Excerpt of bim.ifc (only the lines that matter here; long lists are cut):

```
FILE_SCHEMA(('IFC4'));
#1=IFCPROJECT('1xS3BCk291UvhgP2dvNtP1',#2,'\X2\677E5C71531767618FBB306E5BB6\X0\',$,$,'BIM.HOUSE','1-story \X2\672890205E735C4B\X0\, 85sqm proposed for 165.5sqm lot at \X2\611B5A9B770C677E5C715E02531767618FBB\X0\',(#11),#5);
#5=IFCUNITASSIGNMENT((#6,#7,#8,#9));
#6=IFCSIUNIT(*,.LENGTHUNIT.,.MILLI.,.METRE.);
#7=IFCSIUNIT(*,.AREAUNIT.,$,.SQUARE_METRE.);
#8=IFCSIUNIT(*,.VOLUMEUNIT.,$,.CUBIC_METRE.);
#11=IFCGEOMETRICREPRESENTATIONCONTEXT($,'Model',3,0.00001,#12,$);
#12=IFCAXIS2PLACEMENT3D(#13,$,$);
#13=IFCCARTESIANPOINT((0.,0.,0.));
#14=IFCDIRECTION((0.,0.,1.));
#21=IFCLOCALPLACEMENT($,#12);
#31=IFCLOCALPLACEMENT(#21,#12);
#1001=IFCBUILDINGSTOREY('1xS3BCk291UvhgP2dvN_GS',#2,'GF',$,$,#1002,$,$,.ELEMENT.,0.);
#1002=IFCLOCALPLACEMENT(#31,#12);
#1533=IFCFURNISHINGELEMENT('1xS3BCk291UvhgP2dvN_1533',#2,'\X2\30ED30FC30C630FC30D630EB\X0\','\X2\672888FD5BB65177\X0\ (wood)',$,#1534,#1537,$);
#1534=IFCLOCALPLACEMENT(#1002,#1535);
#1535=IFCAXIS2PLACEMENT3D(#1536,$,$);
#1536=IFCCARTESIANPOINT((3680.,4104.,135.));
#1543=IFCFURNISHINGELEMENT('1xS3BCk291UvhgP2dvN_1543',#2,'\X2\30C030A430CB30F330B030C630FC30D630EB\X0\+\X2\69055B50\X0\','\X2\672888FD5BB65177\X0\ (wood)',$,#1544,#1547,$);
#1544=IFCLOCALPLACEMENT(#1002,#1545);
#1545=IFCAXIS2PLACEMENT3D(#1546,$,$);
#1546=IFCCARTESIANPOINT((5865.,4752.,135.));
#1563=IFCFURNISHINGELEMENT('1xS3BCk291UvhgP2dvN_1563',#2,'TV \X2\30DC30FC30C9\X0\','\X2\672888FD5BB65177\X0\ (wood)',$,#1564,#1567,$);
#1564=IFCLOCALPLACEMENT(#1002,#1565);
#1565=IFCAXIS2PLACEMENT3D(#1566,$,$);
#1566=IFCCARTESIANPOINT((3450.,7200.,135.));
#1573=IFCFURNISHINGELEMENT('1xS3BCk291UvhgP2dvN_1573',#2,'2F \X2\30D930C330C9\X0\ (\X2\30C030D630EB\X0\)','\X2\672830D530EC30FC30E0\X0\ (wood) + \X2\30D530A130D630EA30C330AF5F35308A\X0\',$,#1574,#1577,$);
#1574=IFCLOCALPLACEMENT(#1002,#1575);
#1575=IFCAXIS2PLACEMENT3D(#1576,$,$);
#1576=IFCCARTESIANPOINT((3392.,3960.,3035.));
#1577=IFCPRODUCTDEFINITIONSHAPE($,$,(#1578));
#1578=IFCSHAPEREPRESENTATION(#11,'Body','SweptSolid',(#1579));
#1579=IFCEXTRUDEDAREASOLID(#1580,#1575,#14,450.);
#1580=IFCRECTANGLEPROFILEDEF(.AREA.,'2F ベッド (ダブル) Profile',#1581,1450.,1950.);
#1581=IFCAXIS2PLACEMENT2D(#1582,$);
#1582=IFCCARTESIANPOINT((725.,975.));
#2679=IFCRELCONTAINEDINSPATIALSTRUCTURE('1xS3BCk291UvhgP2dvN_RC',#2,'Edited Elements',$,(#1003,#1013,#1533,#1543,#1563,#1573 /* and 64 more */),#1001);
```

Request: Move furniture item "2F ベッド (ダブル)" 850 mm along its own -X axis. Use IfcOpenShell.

```python
import ifcopenshell
import ifcopenshell.api.geometry
import ifcopenshell.util.placement

model = ifcopenshell.open("bim.ifc")

item = model.by_guid("1xS3BCk291UvhgP2dvN_1573")
matrix = ifcopenshell.util.placement.get_local_placement(item.ObjectPlacement)
matrix[:3, 3] -= matrix[:3, 0] * 850.0
ifcopenshell.api.geometry.edit_object_placement(model, product=item, matrix=matrix, is_si=False)

print(ifcopenshell.util.placement.get_local_placement(item.ObjectPlacement).round(3) + 0.0)

model.write("bim_v2.ifc")
```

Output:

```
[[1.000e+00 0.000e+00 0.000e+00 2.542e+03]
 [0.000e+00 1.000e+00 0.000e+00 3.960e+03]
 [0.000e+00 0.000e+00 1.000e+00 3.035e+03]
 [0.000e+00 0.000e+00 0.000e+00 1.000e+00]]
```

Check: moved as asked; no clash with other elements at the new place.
